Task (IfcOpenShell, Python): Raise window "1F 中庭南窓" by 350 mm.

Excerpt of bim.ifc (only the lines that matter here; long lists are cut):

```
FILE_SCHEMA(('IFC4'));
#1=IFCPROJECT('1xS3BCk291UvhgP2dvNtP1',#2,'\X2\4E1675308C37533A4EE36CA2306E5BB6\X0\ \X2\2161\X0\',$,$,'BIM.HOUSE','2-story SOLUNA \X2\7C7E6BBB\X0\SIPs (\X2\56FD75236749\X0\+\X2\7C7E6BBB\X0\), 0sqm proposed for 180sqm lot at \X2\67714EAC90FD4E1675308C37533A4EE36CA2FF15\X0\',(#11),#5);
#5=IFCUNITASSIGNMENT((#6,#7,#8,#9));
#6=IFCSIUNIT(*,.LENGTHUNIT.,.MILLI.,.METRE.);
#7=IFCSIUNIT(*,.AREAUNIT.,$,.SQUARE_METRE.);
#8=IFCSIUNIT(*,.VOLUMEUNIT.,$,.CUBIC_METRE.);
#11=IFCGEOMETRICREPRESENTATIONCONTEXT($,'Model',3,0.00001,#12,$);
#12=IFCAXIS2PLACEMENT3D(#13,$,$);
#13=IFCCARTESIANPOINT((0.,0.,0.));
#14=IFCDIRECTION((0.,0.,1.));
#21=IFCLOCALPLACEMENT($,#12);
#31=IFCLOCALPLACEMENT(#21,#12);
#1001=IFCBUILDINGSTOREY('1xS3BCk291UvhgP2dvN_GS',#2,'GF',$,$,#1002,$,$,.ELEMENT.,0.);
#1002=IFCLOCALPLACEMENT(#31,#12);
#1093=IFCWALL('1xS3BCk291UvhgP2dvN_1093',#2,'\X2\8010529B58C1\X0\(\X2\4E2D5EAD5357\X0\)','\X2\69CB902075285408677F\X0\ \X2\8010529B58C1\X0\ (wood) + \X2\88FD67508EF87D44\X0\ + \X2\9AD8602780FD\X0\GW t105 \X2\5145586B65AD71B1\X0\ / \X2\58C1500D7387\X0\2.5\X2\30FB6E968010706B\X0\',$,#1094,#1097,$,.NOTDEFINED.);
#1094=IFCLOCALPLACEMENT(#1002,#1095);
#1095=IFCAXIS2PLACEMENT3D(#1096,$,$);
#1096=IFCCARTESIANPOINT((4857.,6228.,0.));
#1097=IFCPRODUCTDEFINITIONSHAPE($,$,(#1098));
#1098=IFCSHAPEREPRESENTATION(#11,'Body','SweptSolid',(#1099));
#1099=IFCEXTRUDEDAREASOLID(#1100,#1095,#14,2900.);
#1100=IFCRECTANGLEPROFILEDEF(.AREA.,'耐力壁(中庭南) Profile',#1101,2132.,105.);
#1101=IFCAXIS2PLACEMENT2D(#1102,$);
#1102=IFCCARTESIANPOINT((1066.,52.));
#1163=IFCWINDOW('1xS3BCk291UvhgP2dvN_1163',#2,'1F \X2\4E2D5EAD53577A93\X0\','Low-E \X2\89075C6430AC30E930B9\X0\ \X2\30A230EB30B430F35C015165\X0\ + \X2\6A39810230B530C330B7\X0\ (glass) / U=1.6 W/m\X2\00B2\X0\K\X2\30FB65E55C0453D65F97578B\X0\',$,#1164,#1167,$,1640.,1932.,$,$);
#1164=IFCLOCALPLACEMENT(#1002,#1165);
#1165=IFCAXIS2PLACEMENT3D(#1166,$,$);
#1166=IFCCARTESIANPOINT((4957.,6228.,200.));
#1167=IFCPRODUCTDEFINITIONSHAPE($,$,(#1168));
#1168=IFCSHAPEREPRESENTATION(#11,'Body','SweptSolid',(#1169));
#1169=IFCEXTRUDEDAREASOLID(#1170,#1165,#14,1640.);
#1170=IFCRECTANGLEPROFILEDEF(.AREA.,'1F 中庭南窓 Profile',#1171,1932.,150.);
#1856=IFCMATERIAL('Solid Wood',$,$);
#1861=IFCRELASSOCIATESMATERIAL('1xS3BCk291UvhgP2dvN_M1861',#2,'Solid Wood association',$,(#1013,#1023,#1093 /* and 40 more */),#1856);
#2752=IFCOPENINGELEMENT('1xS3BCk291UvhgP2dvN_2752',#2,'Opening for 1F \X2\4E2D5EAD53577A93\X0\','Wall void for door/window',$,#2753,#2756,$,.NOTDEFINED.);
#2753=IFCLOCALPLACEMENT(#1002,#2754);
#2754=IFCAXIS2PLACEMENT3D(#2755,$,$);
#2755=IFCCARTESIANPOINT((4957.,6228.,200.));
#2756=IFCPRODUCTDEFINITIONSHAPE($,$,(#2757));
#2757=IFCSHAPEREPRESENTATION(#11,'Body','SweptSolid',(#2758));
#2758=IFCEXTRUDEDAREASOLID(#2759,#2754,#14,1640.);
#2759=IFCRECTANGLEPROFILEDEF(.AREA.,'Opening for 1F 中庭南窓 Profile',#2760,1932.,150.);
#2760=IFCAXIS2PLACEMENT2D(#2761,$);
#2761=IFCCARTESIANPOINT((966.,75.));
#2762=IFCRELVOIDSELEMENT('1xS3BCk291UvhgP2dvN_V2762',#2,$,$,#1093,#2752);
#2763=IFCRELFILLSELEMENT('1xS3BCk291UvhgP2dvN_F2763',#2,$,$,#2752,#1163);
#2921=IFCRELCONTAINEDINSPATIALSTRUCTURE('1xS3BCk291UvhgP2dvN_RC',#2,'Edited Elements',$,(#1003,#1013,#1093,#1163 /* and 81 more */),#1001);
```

```python
import numpy as np
import ifcopenshell
import ifcopenshell.api.geometry
import ifcopenshell.util.placement
import ifcopenshell.util.unit

model = ifcopenshell.open("bim.ifc")
unit_scale = ifcopenshell.util.unit.calculate_unit_scale(model)

window = model.by_guid("1xS3BCk291UvhgP2dvN_1163")
opening = window.FillsVoids[0].RelatingOpeningElement
dz = 0.35 / unit_scale

shift = np.array([0.0, 0.0, dz])
# The window is not placed relative to its opening, so move both.
for product in (opening, window):
    matrix = ifcopenshell.util.placement.get_local_placement(product.ObjectPlacement)
    matrix[:3, 3] += shift
    ifcopenshell.api.geometry.edit_object_placement(model, product=product, matrix=matrix, is_si=False)

print(f"moved by {dz * unit_scale:+.3f} m")

model.write("bim_updated.ifc")
```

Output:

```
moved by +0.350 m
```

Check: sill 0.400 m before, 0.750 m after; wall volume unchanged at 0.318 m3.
